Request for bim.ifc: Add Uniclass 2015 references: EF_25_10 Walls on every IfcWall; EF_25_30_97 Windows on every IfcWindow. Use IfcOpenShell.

First a look at what the model holds.

```python
import ifcopenshell

model = ifcopenshell.open("bim.ifc")
print(model.schema)
print("classifications:", [c.Name for c in model.by_type("IfcClassification")])
for ifc_class in ("IfcDoor", "IfcRoof", "IfcStair", "IfcWall", "IfcWindow"):
    print(ifc_class, len(model.by_type(ifc_class)))
```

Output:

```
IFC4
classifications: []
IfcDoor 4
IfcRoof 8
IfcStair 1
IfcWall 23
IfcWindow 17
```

```python
import ifcopenshell
import ifcopenshell.api.classification

model = ifcopenshell.open("bim.ifc")

system = ifcopenshell.api.classification.add_classification(model, classification="Uniclass 2015")

codes = {
    "IfcWall": ("EF_25_10", "Walls"),
    "IfcWindow": ("EF_25_30_97", "Windows"),
}
for ifc_class, (code, name) in codes.items():
    products = model.by_type(ifc_class)
    ifcopenshell.api.classification.add_reference(
        model, products=products, classification=system, identification=code, name=name
    )
    print(code, len(products))

model.write("bim_edited.ifc")
```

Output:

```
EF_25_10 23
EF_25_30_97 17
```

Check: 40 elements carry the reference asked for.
